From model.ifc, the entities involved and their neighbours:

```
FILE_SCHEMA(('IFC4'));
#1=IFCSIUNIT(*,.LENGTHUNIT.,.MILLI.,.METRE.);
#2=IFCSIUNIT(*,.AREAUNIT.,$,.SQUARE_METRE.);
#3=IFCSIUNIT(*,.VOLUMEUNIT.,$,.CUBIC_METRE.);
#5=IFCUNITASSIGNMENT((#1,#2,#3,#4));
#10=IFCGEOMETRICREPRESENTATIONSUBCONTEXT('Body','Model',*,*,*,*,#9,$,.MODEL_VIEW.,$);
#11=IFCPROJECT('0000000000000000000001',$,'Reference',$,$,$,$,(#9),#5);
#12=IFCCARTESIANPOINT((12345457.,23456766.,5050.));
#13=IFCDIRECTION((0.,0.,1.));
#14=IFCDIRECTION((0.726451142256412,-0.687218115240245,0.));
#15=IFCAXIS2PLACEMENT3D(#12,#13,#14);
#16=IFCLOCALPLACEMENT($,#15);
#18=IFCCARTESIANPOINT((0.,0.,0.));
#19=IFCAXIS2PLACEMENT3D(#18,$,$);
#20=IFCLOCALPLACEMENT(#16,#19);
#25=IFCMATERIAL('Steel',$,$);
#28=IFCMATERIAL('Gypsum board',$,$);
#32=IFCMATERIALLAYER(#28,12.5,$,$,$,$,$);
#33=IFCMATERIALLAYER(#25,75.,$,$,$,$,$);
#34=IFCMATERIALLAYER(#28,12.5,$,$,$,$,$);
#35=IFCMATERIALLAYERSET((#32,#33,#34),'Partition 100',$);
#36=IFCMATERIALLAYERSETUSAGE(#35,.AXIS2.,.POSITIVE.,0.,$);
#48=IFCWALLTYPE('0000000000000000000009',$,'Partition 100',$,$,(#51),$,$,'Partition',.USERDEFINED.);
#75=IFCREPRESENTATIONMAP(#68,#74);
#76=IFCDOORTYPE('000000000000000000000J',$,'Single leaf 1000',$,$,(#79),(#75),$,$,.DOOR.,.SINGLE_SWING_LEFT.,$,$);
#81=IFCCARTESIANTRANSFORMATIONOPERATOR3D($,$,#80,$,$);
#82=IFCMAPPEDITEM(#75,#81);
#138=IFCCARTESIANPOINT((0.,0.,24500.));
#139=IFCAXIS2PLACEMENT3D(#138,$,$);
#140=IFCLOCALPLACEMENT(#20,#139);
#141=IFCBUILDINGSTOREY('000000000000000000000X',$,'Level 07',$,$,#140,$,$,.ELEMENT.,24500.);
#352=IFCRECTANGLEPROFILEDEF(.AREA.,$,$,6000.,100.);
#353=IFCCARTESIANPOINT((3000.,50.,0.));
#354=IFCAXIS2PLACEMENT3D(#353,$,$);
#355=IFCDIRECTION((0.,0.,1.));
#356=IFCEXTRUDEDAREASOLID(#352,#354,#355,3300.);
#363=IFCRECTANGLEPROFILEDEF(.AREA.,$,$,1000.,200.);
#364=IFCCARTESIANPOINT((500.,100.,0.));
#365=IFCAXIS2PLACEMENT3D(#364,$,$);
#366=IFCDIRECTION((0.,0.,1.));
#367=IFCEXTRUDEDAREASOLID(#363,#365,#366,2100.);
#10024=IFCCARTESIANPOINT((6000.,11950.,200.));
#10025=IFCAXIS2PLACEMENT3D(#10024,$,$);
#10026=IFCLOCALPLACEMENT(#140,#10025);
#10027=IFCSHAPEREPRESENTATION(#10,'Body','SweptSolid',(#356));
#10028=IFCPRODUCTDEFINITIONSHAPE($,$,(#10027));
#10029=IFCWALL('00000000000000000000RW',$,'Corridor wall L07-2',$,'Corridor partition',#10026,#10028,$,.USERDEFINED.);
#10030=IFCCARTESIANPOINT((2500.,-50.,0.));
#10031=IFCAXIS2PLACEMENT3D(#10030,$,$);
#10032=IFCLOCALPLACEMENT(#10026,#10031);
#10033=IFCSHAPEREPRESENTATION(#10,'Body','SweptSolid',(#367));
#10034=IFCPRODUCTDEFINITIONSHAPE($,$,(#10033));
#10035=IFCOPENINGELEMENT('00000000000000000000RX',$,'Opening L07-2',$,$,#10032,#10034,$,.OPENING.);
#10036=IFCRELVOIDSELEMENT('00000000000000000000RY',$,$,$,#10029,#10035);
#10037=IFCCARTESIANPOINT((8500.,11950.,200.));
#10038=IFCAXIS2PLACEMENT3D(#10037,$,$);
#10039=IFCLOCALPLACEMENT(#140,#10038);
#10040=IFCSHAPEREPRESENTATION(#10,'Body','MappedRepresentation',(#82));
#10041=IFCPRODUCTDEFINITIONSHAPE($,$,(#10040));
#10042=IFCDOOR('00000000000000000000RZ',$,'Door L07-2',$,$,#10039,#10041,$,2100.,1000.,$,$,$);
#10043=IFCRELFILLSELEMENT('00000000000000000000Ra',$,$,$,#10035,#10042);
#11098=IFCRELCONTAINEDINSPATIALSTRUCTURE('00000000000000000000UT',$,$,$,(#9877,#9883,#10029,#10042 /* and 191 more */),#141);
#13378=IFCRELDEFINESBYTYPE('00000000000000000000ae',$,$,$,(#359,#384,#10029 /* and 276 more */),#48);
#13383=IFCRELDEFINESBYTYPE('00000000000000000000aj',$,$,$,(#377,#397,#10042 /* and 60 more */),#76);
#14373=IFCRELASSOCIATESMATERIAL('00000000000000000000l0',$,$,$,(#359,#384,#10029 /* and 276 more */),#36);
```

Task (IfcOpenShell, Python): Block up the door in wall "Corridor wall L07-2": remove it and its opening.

```python
import ifcopenshell
import ifcopenshell.api.feature
import ifcopenshell.api.root
import ifcopenshell.geom
import ifcopenshell.util.shape

model = ifcopenshell.open("model.ifc")
settings = ifcopenshell.geom.settings()


def volume(element):
    """Net volume in cubic metres, openings subtracted."""
    shape = ifcopenshell.geom.create_shape(settings, element)
    return ifcopenshell.util.shape.get_volume(shape.geometry)


door = model.by_guid("00000000000000000000RZ")
opening = door.FillsVoids[0].RelatingOpeningElement
wall = opening.VoidsElements[0].RelatingBuildingElement
before = volume(wall)

ifcopenshell.api.root.remove_product(model, product=door)
ifcopenshell.api.feature.remove_feature(model, feature=opening)

after = volume(wall)

print(f"wall volume {before:.3f} -> {after:.3f} m3")

model.write("model_updated.ifc")
```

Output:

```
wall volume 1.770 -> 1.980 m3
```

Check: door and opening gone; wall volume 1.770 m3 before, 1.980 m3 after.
